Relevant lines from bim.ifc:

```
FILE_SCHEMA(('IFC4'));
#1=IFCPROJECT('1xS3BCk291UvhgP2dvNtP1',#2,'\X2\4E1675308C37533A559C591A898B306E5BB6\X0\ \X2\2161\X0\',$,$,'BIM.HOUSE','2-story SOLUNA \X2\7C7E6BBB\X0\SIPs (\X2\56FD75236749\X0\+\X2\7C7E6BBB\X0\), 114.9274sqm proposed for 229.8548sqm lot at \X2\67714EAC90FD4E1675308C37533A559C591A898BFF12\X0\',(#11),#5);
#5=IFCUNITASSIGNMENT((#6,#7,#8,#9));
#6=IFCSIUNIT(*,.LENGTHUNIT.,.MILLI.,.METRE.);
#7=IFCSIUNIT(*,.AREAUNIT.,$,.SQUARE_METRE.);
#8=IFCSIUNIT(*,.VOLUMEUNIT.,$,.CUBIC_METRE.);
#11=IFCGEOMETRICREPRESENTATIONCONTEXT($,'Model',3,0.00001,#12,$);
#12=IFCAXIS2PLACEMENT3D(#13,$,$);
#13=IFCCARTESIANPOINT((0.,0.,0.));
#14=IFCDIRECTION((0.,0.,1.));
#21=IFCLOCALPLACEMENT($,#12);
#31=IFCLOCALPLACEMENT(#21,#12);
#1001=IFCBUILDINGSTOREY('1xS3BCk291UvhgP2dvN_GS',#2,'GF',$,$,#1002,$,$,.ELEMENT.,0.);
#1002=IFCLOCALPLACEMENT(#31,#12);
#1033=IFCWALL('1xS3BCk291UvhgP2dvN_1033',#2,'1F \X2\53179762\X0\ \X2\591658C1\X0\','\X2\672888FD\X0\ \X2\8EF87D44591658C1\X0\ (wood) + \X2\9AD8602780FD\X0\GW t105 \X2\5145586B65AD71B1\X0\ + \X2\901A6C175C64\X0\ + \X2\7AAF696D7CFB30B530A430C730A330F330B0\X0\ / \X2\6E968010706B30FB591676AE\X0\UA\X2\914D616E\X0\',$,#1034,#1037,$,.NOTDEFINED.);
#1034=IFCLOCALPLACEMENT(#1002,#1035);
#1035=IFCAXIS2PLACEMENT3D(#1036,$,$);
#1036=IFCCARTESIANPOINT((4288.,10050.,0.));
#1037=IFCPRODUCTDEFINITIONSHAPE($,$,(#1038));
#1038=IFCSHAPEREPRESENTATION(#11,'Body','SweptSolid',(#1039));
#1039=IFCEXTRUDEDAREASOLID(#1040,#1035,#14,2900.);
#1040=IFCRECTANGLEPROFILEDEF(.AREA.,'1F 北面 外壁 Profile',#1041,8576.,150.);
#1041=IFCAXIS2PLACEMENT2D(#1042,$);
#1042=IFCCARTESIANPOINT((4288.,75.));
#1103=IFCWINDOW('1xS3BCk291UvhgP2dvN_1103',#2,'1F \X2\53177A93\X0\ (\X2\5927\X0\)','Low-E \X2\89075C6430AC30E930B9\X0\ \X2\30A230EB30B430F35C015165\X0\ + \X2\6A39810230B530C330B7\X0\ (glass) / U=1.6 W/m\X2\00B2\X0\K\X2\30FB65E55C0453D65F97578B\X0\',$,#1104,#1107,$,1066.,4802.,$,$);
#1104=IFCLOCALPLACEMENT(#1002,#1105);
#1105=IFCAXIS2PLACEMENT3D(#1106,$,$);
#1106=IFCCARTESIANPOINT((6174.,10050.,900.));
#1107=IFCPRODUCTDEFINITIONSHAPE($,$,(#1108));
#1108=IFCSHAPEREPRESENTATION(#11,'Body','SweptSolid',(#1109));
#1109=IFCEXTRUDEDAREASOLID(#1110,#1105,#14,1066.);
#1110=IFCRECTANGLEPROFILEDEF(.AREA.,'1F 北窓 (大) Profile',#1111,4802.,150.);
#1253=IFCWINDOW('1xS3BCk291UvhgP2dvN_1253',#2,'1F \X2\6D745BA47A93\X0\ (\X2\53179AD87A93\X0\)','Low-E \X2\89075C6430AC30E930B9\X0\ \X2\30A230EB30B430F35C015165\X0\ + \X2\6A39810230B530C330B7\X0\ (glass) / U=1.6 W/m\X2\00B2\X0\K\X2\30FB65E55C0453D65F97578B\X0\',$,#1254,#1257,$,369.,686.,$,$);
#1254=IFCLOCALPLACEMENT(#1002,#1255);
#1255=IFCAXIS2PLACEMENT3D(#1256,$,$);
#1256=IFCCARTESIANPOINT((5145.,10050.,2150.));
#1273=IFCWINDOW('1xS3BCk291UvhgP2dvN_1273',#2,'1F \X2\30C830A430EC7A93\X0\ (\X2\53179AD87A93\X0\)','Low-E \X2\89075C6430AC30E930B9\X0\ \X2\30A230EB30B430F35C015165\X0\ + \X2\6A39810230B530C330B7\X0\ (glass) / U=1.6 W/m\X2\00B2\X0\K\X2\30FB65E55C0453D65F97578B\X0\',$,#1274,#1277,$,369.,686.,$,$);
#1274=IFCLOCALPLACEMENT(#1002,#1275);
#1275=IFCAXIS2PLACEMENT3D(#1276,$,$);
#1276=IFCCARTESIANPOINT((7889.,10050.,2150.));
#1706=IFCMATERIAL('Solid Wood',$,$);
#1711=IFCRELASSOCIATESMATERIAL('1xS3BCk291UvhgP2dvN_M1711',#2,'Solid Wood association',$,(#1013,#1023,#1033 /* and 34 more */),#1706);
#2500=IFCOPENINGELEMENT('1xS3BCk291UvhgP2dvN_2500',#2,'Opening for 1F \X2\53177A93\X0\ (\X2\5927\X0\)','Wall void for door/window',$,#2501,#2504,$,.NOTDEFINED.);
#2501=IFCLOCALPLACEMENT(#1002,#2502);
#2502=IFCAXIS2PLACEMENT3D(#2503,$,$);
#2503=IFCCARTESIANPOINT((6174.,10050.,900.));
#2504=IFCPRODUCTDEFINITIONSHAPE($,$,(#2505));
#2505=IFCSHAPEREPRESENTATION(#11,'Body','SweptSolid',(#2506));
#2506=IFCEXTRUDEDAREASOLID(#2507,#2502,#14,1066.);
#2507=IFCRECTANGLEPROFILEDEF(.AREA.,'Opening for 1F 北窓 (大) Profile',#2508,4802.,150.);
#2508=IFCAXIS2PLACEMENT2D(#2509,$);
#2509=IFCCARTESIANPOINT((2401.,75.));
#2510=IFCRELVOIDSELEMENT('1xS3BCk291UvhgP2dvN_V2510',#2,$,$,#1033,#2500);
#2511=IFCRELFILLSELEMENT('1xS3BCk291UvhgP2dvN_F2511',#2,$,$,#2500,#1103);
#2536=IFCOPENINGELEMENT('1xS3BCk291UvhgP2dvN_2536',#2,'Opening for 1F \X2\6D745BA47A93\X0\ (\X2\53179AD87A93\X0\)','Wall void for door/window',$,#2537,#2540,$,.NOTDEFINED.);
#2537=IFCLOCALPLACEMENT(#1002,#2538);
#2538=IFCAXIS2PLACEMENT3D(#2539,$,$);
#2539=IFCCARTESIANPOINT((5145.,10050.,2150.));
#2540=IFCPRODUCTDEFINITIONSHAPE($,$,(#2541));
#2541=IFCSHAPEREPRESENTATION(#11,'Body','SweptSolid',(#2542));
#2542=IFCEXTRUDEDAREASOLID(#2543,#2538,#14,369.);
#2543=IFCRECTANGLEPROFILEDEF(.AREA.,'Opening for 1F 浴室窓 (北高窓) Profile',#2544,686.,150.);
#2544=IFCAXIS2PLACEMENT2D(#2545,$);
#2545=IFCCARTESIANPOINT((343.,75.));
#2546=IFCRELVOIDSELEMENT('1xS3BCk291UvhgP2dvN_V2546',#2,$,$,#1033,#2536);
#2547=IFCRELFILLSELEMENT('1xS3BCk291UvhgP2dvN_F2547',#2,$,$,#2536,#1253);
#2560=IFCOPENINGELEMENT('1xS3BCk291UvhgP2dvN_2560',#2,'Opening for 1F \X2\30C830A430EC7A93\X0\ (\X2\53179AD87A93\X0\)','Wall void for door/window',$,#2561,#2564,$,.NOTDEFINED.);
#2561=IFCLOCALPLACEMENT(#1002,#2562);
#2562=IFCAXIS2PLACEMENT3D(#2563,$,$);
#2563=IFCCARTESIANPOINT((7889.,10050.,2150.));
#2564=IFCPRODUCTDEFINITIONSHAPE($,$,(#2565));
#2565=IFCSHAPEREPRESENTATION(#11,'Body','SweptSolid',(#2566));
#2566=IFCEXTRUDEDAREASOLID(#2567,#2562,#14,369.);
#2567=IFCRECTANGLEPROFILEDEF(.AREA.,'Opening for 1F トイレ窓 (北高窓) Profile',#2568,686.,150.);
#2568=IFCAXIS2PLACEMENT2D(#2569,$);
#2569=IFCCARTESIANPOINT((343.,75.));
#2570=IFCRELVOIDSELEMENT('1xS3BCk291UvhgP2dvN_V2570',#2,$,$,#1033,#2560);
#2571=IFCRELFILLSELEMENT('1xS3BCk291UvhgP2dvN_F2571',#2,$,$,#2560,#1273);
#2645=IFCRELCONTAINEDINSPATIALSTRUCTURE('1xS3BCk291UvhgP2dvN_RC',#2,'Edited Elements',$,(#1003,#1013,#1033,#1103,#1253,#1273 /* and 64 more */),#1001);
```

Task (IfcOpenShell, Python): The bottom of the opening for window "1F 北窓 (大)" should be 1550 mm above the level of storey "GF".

```python
import numpy as np
import ifcopenshell
import ifcopenshell.api.geometry
import ifcopenshell.geom
import ifcopenshell.util.element
import ifcopenshell.util.placement
import ifcopenshell.util.shape
import ifcopenshell.util.unit

model = ifcopenshell.open("bim.ifc")
unit_scale = ifcopenshell.util.unit.calculate_unit_scale(model)

window = model.by_guid("1xS3BCk291UvhgP2dvN_1103")
opening = window.FillsVoids[0].RelatingOpeningElement
storey = ifcopenshell.util.element.get_container(window, ifc_class="IfcBuildingStorey")
level = ifcopenshell.util.placement.get_local_placement(storey.ObjectPlacement)[2, 3]

# The opening's origin need not be at the sill, so measure its lowest point.
shape = ifcopenshell.geom.create_shape(ifcopenshell.geom.settings(), opening)
bottom = ifcopenshell.util.shape.get_shape_bottom_elevation(shape, shape.geometry) / unit_scale
dz = level + 1550.0 - bottom

shift = np.array([0.0, 0.0, dz])
# The window is not placed relative to its opening, so move both.
for product in (opening, window):
    matrix = ifcopenshell.util.placement.get_local_placement(product.ObjectPlacement)
    matrix[:3, 3] += shift
    ifcopenshell.api.geometry.edit_object_placement(model, product=product, matrix=matrix, is_si=False)

print(f"moved by {dz * unit_scale:+.3f} m")

model.write("bim_v2.ifc")
```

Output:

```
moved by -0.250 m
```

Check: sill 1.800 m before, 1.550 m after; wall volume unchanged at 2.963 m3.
